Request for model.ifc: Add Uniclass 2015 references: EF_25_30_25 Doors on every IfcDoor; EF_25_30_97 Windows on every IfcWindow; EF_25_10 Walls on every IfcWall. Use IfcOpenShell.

First a look at what the model holds.

```python
import ifcopenshell

model = ifcopenshell.open("model.ifc")
print(model.schema)
print("classifications:", [c.Name for c in model.by_type("IfcClassification")])
for ifc_class in ("IfcDoor", "IfcRoof", "IfcStair", "IfcWall", "IfcWindow"):
    print(ifc_class, len(model.by_type(ifc_class)))
```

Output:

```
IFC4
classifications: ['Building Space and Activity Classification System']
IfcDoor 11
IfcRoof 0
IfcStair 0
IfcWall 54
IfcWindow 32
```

```python
import ifcopenshell
import ifcopenshell.api.classification

model = ifcopenshell.open("model.ifc")

system = ifcopenshell.api.classification.add_classification(model, classification="Uniclass 2015")

codes = {
    "IfcDoor": ("EF_25_30_25", "Doors"),
    "IfcWindow": ("EF_25_30_97", "Windows"),
    "IfcWall": ("EF_25_10", "Walls"),
}
for ifc_class, (code, name) in codes.items():
    products = model.by_type(ifc_class)
    ifcopenshell.api.classification.add_reference(
        model, products=products, classification=system, identification=code, name=name
    )
    print(code, len(products))

model.write("model_v2.ifc")
```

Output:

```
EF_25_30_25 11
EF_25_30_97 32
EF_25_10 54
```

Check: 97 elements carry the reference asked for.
